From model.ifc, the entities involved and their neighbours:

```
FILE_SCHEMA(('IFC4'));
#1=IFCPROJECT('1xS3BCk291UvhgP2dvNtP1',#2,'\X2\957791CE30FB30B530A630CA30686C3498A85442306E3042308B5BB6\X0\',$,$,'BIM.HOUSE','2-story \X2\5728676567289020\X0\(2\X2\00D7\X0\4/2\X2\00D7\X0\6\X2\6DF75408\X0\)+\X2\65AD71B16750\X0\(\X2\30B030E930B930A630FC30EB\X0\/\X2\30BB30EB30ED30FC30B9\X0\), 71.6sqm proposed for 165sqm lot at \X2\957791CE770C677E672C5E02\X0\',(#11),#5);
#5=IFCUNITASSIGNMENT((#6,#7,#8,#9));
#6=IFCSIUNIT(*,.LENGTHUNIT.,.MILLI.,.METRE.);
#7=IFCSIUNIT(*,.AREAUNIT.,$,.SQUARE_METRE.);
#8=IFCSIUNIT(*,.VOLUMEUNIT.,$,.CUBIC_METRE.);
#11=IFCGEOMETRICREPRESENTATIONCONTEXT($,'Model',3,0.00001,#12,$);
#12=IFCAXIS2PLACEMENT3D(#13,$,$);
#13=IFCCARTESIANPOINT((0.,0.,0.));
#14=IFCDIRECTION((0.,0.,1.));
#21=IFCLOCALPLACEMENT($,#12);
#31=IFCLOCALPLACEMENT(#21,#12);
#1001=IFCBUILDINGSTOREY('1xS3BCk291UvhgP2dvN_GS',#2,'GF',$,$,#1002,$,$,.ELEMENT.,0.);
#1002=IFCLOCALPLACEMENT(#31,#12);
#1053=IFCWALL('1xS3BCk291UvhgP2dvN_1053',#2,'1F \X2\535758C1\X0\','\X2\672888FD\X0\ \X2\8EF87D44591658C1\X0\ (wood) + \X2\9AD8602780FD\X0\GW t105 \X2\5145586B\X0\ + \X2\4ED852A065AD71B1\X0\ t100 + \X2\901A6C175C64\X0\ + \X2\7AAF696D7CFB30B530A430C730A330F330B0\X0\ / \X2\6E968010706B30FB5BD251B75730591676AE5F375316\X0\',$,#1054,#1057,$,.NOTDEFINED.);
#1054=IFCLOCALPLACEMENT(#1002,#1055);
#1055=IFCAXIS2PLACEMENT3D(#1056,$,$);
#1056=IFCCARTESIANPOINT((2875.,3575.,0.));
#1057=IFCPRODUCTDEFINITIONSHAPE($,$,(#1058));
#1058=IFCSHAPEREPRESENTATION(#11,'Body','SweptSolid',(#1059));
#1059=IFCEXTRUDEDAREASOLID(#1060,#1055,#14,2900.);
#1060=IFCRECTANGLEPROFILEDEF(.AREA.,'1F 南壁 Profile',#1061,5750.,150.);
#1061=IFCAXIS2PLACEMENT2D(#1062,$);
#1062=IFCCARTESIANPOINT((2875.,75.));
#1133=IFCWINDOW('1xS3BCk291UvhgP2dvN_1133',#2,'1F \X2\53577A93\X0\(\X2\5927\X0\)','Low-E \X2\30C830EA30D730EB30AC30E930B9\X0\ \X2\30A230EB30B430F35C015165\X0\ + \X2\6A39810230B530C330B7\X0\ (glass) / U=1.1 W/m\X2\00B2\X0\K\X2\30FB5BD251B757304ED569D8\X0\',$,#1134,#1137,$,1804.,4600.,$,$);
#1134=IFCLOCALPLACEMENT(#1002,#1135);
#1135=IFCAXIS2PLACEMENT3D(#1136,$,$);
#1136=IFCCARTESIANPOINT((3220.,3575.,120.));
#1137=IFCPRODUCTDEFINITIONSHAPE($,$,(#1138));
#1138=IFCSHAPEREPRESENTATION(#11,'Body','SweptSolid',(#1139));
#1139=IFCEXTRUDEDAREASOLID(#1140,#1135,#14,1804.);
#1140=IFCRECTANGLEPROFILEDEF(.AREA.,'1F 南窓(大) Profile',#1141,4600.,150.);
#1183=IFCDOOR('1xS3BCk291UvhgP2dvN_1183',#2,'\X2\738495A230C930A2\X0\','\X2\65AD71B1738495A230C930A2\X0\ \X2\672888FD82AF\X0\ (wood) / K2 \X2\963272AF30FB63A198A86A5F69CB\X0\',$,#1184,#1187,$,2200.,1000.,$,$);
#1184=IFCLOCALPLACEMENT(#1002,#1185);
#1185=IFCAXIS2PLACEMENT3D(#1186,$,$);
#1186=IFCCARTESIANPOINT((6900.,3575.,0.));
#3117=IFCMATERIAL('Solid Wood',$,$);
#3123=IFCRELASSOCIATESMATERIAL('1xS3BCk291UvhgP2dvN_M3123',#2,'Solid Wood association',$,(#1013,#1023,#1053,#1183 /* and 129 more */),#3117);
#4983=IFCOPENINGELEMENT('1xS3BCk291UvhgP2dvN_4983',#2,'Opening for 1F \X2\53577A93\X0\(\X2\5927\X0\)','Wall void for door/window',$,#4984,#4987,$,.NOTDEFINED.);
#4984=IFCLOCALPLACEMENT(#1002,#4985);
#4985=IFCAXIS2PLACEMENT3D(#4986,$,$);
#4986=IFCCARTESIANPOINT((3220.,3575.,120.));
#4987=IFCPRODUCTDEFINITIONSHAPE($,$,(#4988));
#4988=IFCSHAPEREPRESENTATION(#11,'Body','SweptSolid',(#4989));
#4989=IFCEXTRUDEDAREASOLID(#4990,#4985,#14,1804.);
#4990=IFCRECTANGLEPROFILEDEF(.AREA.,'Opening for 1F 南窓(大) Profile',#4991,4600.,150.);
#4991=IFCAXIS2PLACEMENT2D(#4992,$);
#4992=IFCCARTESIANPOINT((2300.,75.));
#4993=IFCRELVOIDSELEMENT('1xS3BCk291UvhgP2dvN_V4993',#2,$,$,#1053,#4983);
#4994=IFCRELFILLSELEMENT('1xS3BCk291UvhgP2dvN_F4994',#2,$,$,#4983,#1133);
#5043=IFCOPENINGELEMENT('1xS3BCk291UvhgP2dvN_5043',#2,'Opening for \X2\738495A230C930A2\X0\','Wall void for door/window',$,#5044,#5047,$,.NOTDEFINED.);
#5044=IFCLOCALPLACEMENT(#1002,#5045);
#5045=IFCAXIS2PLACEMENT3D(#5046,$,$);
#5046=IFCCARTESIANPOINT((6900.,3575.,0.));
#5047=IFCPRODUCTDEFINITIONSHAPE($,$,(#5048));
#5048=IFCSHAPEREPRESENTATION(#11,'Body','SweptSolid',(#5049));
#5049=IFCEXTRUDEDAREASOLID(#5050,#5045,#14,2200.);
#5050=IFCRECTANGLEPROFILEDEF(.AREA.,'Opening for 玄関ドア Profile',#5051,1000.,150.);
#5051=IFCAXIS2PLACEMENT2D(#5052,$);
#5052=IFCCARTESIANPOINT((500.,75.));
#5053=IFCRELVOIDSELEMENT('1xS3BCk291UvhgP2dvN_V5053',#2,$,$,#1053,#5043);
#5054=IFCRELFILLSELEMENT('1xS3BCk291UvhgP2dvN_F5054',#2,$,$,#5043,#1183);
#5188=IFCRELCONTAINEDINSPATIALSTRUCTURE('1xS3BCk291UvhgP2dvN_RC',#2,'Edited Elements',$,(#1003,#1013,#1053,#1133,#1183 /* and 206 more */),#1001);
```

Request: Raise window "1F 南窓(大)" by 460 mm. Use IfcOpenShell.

```python
import numpy as np
import ifcopenshell
import ifcopenshell.api.geometry
import ifcopenshell.util.placement
import ifcopenshell.util.unit

model = ifcopenshell.open("model.ifc")
unit_scale = ifcopenshell.util.unit.calculate_unit_scale(model)

window = model.by_guid("1xS3BCk291UvhgP2dvN_1133")
opening = window.FillsVoids[0].RelatingOpeningElement
dz = 0.46 / unit_scale

shift = np.array([0.0, 0.0, dz])
# The window is not placed relative to its opening, so move both.
for product in (opening, window):
    matrix = ifcopenshell.util.placement.get_local_placement(product.ObjectPlacement)
    matrix[:3, 3] += shift
    ifcopenshell.api.geometry.edit_object_placement(model, product=product, matrix=matrix, is_si=False)

print(f"moved by {dz * unit_scale:+.3f} m")

model.write("model_v2.ifc")
```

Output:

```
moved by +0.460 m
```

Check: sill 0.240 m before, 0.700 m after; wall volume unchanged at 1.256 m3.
